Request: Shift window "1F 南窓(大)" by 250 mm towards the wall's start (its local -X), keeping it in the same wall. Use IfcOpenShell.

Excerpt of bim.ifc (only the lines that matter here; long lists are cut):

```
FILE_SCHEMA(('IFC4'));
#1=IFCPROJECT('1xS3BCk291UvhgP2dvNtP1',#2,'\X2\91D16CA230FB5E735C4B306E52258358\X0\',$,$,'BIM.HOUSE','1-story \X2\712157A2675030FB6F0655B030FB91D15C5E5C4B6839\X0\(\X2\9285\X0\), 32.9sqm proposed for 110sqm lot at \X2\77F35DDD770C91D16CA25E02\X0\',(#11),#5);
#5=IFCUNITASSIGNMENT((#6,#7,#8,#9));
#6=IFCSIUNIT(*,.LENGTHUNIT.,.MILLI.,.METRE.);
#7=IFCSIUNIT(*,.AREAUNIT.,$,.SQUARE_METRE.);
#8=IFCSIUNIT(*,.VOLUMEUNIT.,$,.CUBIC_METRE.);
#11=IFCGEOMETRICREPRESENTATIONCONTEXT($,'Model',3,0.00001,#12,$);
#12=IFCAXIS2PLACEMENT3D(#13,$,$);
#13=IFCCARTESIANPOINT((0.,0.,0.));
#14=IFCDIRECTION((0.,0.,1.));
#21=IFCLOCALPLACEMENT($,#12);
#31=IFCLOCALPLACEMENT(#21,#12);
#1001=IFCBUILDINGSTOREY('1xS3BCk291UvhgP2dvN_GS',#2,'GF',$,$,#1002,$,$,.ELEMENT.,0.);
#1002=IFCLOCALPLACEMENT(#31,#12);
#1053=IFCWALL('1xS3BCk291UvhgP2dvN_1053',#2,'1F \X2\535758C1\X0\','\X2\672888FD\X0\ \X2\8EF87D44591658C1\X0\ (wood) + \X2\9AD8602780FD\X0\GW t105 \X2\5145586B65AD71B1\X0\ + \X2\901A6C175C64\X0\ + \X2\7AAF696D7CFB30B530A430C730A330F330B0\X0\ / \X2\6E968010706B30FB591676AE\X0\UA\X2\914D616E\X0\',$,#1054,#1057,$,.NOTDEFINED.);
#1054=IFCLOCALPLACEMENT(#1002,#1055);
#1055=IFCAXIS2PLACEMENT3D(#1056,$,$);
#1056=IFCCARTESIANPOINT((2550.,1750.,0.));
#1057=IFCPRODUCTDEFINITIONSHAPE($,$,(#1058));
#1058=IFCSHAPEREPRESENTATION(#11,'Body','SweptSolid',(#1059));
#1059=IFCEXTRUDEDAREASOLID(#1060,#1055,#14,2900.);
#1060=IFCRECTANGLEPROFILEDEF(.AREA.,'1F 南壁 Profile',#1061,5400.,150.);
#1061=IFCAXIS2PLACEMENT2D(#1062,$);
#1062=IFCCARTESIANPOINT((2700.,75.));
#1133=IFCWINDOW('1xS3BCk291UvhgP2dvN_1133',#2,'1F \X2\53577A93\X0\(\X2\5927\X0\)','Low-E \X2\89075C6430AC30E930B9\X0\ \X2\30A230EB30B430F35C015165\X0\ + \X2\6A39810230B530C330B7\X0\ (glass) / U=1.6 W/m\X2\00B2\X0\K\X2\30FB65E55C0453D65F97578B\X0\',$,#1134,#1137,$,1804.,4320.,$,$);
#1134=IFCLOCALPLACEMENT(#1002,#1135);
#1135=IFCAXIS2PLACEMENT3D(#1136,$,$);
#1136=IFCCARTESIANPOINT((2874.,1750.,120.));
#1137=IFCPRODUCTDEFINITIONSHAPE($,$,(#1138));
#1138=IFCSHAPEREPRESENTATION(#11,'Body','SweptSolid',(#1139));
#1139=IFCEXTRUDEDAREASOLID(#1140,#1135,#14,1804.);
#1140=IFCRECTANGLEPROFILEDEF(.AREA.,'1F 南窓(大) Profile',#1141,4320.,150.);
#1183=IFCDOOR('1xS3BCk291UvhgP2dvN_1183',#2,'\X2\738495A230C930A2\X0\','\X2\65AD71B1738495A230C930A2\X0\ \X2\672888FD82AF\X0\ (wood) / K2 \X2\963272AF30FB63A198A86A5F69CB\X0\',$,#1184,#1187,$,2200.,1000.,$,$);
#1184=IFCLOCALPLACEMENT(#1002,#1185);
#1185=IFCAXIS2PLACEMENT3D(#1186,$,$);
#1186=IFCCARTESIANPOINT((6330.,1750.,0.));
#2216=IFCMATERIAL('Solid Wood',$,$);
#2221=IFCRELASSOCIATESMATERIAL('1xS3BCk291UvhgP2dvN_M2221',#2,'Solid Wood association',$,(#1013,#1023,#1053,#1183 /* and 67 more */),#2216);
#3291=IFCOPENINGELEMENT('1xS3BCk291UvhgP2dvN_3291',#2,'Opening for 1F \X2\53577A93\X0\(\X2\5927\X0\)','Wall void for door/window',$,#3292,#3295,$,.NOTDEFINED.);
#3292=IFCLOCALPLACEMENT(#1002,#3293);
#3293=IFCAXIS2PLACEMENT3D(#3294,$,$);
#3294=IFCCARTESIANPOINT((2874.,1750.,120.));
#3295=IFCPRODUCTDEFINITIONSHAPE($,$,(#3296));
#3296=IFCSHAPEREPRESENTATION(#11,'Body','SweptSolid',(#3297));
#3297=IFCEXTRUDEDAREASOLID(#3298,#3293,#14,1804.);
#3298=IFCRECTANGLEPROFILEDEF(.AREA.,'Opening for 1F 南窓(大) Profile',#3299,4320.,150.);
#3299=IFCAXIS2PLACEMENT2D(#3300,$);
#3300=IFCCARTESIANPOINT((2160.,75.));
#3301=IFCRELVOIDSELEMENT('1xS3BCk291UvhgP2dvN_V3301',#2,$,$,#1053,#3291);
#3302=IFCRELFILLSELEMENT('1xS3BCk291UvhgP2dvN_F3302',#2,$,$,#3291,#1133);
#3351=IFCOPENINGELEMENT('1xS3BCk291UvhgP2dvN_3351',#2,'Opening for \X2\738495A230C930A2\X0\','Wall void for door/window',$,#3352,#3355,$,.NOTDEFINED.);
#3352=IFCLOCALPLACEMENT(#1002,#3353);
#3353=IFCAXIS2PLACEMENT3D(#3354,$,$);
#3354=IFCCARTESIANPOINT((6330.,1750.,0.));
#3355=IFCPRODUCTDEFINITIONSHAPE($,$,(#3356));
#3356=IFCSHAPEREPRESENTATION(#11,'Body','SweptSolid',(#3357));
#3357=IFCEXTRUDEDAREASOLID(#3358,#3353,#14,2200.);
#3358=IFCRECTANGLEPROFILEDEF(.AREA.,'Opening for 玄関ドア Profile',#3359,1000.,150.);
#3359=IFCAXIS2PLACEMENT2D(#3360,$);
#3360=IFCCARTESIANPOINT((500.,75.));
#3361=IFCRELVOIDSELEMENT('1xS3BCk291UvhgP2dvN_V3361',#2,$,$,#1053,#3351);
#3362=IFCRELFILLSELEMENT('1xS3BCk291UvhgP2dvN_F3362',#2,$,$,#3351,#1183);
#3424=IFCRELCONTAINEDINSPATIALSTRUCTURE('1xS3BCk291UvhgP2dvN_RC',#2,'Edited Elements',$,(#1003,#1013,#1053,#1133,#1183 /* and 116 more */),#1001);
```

```python
import ifcopenshell
import ifcopenshell.api.geometry
import ifcopenshell.util.placement
import ifcopenshell.util.unit

model = ifcopenshell.open("bim.ifc")
unit_scale = ifcopenshell.util.unit.calculate_unit_scale(model)

window = model.by_guid("1xS3BCk291UvhgP2dvN_1133")
opening = window.FillsVoids[0].RelatingOpeningElement
wall = opening.VoidsElements[0].RelatingBuildingElement

wall_matrix = ifcopenshell.util.placement.get_local_placement(wall.ObjectPlacement)
shift = wall_matrix[:3, 0] * -0.25 / unit_scale
before = ifcopenshell.util.placement.get_local_placement(window.ObjectPlacement)[:3, 3].copy()

# The window is not placed relative to its opening, so move both.
for product in (opening, window):
    matrix = ifcopenshell.util.placement.get_local_placement(product.ObjectPlacement)
    matrix[:3, 3] += shift
    ifcopenshell.api.geometry.edit_object_placement(model, product=product, matrix=matrix, is_si=False)

after = ifcopenshell.util.placement.get_local_placement(window.ObjectPlacement)[:3, 3]
print("window moved by", (after - before).round(3) + 0.0)

model.write("bim_updated.ifc")
```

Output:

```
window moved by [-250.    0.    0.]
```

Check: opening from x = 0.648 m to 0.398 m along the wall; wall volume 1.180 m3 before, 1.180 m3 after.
